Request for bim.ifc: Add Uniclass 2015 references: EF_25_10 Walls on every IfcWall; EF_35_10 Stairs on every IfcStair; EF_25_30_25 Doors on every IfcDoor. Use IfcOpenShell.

First a look at what the model holds.

```python
import ifcopenshell

model = ifcopenshell.open("bim.ifc")
print(model.schema)
print("classifications:", [c.Name for c in model.by_type("IfcClassification")])
for ifc_class in ("IfcDoor", "IfcRoof", "IfcStair", "IfcWall", "IfcWindow"):
    print(ifc_class, len(model.by_type(ifc_class)))
```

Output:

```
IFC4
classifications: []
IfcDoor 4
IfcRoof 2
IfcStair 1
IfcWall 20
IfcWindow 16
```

```python
import ifcopenshell
import ifcopenshell.api.classification

model = ifcopenshell.open("bim.ifc")

system = ifcopenshell.api.classification.add_classification(model, classification="Uniclass 2015")

codes = {
    "IfcWall": ("EF_25_10", "Walls"),
    "IfcStair": ("EF_35_10", "Stairs"),
    "IfcDoor": ("EF_25_30_25", "Doors"),
}
for ifc_class, (code, name) in codes.items():
    products = model.by_type(ifc_class)
    ifcopenshell.api.classification.add_reference(
        model, products=products, classification=system, identification=code, name=name
    )
    print(code, len(products))

model.write("bim_v2.ifc")
```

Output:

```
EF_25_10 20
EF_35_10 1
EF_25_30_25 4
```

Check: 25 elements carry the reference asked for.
